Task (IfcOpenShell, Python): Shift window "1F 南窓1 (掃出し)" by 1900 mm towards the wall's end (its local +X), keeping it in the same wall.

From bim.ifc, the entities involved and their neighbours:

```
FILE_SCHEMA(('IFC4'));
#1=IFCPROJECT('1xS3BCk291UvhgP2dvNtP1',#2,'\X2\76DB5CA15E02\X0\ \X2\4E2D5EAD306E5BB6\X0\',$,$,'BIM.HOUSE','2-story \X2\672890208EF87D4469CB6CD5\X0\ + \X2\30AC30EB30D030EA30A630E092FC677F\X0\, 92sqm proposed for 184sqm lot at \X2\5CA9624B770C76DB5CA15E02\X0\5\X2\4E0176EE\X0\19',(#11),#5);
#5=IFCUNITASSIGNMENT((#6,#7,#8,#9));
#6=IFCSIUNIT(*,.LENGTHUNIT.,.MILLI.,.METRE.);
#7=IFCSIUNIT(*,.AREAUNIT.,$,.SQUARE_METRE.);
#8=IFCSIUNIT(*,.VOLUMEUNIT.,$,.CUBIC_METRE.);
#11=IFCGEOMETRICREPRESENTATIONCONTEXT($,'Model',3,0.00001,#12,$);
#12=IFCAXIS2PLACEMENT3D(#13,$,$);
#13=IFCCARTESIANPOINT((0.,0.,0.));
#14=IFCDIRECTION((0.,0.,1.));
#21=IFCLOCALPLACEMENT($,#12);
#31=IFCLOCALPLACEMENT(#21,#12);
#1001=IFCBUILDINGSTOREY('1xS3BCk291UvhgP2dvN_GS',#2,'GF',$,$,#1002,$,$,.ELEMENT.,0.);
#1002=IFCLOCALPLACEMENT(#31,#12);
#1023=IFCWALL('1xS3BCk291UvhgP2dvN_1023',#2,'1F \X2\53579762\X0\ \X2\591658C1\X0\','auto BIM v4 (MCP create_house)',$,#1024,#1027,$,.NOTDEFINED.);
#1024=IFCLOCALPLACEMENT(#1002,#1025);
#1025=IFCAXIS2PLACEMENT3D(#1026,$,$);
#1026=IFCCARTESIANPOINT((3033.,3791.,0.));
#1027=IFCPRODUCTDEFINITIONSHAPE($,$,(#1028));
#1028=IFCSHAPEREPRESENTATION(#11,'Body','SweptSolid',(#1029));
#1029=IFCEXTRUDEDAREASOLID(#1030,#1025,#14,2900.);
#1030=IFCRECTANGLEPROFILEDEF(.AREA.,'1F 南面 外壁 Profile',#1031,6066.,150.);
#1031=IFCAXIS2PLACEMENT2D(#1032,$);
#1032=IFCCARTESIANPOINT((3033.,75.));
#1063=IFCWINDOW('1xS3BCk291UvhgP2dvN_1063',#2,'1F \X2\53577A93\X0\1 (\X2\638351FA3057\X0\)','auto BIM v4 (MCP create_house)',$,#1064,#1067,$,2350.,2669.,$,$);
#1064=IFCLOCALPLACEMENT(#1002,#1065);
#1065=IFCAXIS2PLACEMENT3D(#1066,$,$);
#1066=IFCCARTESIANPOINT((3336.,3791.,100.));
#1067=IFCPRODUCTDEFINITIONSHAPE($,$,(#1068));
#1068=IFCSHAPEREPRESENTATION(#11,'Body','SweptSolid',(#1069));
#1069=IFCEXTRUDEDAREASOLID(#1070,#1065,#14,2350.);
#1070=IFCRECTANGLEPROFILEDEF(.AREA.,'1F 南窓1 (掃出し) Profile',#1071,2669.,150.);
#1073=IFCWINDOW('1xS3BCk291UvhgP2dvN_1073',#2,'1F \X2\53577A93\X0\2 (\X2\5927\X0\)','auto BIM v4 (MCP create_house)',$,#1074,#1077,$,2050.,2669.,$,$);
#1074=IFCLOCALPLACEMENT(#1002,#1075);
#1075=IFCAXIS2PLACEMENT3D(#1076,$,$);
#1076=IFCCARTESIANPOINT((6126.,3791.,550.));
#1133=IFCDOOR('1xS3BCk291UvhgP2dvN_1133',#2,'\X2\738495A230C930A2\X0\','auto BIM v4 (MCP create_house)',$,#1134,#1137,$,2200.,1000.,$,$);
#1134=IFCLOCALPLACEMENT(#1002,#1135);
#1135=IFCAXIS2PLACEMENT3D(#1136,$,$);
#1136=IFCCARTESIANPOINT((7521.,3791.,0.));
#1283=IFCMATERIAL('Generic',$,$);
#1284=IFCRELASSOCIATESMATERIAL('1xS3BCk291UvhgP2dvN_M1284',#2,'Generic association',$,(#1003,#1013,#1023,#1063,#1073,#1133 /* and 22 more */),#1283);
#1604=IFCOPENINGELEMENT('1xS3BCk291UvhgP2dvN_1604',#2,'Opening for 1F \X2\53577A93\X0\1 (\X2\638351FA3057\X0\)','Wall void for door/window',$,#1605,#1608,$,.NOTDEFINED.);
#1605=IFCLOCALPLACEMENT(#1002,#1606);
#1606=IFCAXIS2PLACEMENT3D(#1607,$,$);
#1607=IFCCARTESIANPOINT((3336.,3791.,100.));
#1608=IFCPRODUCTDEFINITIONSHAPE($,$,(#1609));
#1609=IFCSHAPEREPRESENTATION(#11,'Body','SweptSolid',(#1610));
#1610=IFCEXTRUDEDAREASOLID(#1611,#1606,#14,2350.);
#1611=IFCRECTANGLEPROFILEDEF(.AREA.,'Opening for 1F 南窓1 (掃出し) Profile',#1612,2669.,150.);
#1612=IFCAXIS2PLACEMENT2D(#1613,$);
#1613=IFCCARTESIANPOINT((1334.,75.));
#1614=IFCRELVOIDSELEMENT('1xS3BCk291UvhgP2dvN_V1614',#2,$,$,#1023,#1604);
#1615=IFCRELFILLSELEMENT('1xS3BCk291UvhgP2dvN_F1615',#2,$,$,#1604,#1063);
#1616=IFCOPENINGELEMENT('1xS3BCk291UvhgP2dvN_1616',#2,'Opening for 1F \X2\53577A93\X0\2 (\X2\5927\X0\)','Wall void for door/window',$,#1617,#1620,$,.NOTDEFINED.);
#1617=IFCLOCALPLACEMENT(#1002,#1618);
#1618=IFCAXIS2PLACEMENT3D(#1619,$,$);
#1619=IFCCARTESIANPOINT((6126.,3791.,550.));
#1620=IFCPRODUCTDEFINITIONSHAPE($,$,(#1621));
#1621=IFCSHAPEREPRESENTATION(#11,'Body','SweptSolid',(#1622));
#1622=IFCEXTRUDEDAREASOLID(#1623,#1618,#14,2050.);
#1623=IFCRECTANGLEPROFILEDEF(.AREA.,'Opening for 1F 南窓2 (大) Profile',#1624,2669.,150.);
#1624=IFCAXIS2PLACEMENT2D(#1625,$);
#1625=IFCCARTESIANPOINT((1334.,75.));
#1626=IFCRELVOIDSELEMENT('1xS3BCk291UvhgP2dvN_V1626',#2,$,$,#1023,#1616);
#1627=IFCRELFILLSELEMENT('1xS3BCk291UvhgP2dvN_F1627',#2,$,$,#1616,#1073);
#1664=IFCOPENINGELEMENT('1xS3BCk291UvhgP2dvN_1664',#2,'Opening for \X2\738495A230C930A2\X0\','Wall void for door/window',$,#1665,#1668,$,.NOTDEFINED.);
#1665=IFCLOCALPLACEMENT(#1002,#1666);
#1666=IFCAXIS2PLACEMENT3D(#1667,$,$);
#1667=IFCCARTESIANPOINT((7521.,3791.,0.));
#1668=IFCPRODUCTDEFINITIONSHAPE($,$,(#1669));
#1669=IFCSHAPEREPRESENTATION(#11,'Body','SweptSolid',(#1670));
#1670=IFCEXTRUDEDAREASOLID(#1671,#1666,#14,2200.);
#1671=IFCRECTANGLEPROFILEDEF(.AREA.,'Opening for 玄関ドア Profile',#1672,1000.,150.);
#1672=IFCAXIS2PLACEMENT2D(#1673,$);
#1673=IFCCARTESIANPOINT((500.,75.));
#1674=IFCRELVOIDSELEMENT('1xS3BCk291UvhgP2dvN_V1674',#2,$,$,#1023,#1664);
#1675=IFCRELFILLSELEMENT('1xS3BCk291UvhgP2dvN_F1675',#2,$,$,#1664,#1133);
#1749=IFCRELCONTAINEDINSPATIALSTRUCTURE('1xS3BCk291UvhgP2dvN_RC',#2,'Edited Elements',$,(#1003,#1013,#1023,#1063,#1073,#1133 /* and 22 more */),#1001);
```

```python
import ifcopenshell
import ifcopenshell.api.geometry
import ifcopenshell.util.placement

model = ifcopenshell.open("bim.ifc")

window = model.by_guid("1xS3BCk291UvhgP2dvN_1063")
opening = window.FillsVoids[0].RelatingOpeningElement
wall = opening.VoidsElements[0].RelatingBuildingElement

wall_matrix = ifcopenshell.util.placement.get_local_placement(wall.ObjectPlacement)
shift = wall_matrix[:3, 0] * 1900.0
before = ifcopenshell.util.placement.get_local_placement(window.ObjectPlacement)[:3, 3].copy()

# The window is not placed relative to its opening, so move both.
for product in (opening, window):
    matrix = ifcopenshell.util.placement.get_local_placement(product.ObjectPlacement)
    matrix[:3, 3] += shift
    ifcopenshell.api.geometry.edit_object_placement(model, product=product, matrix=matrix, is_si=False)

after = ifcopenshell.util.placement.get_local_placement(window.ObjectPlacement)[:3, 3]
print("window moved by", (after - before).round(3) + 0.0)

model.write("bim_edited.ifc")
```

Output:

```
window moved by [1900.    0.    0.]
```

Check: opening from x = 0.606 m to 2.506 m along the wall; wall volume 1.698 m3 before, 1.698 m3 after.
